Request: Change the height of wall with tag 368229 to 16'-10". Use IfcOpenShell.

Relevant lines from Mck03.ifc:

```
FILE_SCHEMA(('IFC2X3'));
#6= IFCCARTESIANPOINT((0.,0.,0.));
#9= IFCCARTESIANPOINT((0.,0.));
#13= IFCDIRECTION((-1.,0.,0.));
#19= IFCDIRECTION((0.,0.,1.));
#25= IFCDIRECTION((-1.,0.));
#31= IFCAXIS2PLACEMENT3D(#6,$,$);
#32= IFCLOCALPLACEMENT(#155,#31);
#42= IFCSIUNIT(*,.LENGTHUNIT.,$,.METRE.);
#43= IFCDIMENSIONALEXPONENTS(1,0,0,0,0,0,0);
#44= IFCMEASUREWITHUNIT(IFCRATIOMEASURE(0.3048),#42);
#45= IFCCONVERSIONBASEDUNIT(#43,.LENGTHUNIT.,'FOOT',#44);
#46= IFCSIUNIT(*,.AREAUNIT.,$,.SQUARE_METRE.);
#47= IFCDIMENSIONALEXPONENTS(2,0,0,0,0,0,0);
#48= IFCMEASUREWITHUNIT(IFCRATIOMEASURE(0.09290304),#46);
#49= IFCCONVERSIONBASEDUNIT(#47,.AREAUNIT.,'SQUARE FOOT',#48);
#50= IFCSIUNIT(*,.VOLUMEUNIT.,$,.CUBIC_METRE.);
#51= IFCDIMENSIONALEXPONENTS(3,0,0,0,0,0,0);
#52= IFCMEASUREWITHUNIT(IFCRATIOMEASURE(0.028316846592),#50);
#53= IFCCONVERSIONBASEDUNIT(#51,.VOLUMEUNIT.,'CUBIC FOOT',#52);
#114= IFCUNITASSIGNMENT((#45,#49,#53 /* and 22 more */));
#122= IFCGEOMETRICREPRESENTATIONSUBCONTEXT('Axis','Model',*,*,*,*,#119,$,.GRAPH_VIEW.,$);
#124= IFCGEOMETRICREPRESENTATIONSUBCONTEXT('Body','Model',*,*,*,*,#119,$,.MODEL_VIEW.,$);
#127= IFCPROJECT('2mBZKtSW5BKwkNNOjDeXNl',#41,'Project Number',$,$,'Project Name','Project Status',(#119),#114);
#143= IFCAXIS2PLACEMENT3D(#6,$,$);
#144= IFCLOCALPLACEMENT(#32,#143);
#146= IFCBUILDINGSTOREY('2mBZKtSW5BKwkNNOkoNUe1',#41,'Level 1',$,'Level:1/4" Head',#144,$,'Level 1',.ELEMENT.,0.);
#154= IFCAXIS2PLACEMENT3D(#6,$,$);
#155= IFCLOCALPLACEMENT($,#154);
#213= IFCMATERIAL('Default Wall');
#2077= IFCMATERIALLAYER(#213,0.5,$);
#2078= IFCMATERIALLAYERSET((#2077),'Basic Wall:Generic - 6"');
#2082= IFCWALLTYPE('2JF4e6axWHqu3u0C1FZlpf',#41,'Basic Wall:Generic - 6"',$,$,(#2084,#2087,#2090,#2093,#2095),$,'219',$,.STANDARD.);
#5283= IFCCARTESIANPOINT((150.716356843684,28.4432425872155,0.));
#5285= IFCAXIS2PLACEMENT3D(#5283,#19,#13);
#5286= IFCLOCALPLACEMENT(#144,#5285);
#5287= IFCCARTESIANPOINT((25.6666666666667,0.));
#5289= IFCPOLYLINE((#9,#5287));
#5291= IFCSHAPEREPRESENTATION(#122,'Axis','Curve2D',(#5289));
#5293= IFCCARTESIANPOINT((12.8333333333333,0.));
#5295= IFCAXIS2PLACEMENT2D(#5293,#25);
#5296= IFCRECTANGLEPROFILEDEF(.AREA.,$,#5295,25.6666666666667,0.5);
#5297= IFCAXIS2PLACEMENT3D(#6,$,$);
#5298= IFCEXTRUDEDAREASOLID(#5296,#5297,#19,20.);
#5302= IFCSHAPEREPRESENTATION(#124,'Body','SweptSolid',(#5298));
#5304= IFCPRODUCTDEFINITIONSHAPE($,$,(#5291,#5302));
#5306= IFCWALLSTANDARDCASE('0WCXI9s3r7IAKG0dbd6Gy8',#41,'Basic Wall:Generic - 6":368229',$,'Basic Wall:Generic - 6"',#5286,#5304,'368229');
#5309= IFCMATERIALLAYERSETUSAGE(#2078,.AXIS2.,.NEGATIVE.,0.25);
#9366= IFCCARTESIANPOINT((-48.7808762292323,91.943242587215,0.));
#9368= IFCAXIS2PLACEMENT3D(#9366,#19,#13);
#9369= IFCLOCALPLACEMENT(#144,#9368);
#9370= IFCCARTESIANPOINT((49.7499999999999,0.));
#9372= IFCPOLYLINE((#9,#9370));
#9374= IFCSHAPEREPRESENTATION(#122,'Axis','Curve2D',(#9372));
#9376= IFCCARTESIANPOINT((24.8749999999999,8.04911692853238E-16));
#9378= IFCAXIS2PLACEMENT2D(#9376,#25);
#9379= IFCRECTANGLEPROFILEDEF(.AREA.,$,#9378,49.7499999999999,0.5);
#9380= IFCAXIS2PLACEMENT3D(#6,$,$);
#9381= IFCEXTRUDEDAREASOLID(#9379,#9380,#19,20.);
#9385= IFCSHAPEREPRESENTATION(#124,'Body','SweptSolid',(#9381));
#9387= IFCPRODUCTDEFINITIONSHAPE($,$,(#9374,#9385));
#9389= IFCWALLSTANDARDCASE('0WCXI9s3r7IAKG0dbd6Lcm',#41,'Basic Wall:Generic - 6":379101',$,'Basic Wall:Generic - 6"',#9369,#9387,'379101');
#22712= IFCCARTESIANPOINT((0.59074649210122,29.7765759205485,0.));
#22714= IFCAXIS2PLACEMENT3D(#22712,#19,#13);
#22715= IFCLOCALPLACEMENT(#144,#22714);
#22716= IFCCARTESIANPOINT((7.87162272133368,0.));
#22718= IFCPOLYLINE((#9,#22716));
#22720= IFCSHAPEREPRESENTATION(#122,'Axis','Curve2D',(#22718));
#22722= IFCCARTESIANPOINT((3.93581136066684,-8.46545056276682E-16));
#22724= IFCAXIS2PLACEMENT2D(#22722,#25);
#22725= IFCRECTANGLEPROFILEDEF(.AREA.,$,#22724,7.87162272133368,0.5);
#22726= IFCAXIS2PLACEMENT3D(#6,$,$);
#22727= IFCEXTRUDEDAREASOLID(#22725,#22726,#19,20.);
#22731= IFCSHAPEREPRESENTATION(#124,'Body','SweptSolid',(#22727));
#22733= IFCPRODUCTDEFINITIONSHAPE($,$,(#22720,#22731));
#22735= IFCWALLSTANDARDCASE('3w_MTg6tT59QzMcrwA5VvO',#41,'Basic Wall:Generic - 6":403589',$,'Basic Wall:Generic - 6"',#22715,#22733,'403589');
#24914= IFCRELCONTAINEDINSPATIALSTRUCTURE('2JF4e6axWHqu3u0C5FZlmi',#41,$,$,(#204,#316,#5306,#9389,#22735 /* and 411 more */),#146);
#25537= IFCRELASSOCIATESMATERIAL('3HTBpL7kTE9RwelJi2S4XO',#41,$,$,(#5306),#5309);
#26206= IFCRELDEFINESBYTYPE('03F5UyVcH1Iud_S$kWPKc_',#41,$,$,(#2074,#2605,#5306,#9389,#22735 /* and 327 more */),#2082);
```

```python
import ifcopenshell
import ifcopenshell.geom
import ifcopenshell.util.representation
import ifcopenshell.util.shape
import ifcopenshell.util.unit

model = ifcopenshell.open("Mck03.ifc")
unit_scale = ifcopenshell.util.unit.calculate_unit_scale(model)
settings = ifcopenshell.geom.settings()


def volume(element):
    """Net volume in cubic metres, openings subtracted."""
    shape = ifcopenshell.geom.create_shape(settings, element)
    return ifcopenshell.util.shape.get_volume(shape.geometry)


wall = model.by_guid("0WCXI9s3r7IAKG0dbd6Gy8")
before = volume(wall)

body = ifcopenshell.util.representation.get_representation(wall, "Model", "Body")
solid = body.Items[0]
old_height = solid.Depth
solid.Depth = 202 * 0.0254 / unit_scale
after = volume(wall)

print(f"height {old_height:g} -> {solid.Depth:g}, volume {before:.3f} -> {after:.3f} m3")

model.write("Mck03_edited.ifc")
```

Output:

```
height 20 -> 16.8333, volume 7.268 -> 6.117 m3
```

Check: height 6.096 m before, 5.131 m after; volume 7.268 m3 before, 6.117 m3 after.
